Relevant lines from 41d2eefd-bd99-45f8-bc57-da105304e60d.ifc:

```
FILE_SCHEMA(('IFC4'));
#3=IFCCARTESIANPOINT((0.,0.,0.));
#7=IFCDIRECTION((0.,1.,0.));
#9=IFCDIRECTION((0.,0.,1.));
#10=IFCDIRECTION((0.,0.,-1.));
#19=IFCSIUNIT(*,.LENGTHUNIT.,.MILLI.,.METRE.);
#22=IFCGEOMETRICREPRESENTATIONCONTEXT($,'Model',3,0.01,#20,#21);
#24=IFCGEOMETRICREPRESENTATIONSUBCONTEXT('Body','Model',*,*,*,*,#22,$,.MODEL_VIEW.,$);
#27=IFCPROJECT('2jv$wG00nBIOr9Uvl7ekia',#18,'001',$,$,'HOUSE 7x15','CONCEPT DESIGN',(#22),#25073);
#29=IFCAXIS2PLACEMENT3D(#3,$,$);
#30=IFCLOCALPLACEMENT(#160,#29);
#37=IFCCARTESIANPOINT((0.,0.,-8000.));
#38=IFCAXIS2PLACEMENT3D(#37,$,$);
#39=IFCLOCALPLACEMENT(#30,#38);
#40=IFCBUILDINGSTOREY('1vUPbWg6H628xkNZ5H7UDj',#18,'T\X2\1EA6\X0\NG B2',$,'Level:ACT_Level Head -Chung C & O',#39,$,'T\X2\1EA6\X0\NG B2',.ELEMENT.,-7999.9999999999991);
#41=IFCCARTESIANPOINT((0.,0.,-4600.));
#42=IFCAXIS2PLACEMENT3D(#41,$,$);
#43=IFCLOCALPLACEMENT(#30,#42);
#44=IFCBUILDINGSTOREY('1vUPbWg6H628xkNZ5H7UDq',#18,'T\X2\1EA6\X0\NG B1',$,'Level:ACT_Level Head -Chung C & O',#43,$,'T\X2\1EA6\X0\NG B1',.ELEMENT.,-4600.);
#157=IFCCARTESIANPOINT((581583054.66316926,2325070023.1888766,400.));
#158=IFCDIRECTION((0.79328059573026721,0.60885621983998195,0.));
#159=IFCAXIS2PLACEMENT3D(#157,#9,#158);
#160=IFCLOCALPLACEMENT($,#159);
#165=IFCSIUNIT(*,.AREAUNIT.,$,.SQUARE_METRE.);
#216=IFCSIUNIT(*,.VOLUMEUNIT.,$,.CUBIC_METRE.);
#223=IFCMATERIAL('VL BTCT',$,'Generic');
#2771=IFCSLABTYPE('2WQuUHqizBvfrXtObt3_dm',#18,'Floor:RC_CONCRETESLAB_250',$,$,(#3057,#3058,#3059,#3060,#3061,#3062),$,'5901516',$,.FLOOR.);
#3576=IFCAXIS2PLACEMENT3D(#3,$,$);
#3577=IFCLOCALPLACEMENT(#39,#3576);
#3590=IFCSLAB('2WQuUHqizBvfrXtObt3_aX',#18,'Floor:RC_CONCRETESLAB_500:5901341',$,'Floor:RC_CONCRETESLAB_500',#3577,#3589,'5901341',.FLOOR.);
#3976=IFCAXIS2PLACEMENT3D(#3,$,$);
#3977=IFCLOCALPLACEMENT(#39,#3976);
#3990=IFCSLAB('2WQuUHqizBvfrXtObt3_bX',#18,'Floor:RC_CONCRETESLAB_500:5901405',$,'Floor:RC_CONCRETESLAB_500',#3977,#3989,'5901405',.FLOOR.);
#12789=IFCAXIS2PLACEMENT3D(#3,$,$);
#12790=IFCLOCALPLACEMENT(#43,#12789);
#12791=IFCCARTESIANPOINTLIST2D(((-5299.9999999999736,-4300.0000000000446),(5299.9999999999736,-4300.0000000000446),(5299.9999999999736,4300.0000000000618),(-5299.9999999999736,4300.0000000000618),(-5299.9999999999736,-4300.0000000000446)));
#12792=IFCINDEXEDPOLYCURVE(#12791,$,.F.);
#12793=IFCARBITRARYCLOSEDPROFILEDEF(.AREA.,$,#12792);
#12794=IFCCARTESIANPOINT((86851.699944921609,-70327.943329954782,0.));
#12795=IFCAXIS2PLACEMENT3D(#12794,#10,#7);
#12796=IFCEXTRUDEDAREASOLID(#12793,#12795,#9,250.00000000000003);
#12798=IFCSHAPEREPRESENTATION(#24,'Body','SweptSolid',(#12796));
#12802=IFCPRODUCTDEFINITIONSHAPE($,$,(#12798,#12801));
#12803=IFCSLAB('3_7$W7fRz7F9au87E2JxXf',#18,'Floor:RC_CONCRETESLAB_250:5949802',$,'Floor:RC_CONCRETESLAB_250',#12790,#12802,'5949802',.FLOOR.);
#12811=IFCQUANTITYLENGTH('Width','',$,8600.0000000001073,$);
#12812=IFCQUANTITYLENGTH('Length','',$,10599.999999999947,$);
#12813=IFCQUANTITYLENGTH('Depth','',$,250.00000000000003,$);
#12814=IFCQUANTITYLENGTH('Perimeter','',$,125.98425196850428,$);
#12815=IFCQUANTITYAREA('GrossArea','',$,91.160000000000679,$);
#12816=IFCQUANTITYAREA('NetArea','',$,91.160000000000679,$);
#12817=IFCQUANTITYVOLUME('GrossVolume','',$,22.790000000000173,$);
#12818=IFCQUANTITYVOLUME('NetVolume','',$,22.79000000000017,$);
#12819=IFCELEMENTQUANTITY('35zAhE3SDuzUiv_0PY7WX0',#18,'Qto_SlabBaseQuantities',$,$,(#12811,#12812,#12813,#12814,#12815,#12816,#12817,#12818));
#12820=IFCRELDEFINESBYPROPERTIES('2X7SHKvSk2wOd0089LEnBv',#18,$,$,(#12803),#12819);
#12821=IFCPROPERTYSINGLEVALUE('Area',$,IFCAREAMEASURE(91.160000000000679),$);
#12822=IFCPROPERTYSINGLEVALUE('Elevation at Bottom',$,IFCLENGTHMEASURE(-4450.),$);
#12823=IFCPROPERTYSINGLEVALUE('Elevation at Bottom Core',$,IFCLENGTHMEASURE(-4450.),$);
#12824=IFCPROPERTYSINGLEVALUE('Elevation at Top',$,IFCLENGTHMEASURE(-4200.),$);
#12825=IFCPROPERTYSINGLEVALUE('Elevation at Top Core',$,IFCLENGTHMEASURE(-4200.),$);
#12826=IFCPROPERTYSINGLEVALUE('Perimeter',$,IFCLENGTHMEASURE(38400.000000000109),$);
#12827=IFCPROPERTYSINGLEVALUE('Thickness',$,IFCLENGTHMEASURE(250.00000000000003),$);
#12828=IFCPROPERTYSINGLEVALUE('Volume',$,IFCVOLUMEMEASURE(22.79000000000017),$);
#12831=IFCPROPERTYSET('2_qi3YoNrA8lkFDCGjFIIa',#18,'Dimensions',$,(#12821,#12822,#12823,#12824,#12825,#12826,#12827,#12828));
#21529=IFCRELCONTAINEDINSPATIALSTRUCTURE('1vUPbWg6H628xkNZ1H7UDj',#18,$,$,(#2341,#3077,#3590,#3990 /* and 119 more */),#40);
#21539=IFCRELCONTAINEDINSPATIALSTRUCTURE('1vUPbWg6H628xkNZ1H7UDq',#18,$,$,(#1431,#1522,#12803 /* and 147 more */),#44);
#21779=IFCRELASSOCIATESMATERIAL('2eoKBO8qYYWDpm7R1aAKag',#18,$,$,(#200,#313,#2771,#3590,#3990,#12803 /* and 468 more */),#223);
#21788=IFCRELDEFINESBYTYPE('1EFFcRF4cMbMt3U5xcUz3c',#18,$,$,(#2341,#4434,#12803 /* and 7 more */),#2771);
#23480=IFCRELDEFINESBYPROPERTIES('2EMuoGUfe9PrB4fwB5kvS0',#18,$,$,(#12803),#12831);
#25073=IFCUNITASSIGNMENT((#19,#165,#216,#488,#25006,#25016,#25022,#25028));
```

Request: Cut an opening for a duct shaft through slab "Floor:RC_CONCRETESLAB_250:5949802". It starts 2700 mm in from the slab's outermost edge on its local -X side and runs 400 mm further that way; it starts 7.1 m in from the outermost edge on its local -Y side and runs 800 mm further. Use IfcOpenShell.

```python
import numpy as np
import ifcopenshell
import ifcopenshell.api.feature
import ifcopenshell.api.geometry
import ifcopenshell.api.pset
import ifcopenshell.api.root
import ifcopenshell.geom
import ifcopenshell.util.element
import ifcopenshell.util.placement
import ifcopenshell.util.representation
import ifcopenshell.util.shape
import ifcopenshell.util.unit

model = ifcopenshell.open("41d2eefd-bd99-45f8-bc57-da105304e60d.ifc")
unit_scale = ifcopenshell.util.unit.calculate_unit_scale(model)
area_scale = ifcopenshell.util.unit.calculate_unit_scale(model, "AREAUNIT")
volume_scale = ifcopenshell.util.unit.calculate_unit_scale(model, "VOLUMEUNIT")
settings = ifcopenshell.geom.settings()


def volume(element):
    """Net volume in cubic metres, openings subtracted."""
    shape = ifcopenshell.geom.create_shape(settings, element)
    return ifcopenshell.util.shape.get_volume(shape.geometry)


slab = model.by_guid("3_7$W7fRz7F9au87E2JxXf")
before = volume(slab)

# Extent in the slab's own axes, in metres. The edges named are its -X and -Y sides.
slab_shape = ifcopenshell.geom.create_shape(settings, slab)
vertices = ifcopenshell.util.shape.get_vertices(slab_shape.geometry)
x_min, y_min, bottom = vertices.min(axis=0)
top = vertices[:, 2].max()

opening = ifcopenshell.api.root.create_entity(model, ifc_class="IfcOpeningElement", name="Duct shaft opening", predefined_type="OPENING")
context = ifcopenshell.util.representation.get_context(model, "Model", "Body", "MODEL_VIEW")
width, depth = 0.4, 0.8
outline = [(0.0, 0.0), (width, 0.0), (width, depth), (0.0, depth), (0.0, 0.0)]
# Overshoot both faces by 50 mm so the cut is clean.
shape = ifcopenshell.api.geometry.add_slab_representation(
    model, context=context, depth=top - bottom + 0.1, polyline=outline
)
ifcopenshell.api.geometry.assign_representation(model, product=opening, representation=shape)

matrix = ifcopenshell.util.placement.get_local_placement(slab.ObjectPlacement)
matrix[:, 3] = matrix @ np.append(np.array([x_min + 2.7, y_min + 7.1, bottom - 0.05]) / unit_scale, 1.0)
ifcopenshell.api.geometry.edit_object_placement(model, product=opening, matrix=matrix, is_si=False)
ifcopenshell.api.feature.add_feature(model, feature=opening, element=slab)

after = volume(slab)

# Update the slab's stored quantities.
qto = model.by_id(ifcopenshell.util.element.get_pset(slab, "Qto_SlabBaseQuantities", should_inherit=False)["id"])
ifcopenshell.api.pset.edit_qto(model, qto=qto, properties={
    "NetArea": after / (top - bottom) / area_scale,
    "NetVolume": after / volume_scale,
})
pset = model.by_id(ifcopenshell.util.element.get_pset(slab, "Dimensions", should_inherit=False)["id"])
ifcopenshell.api.pset.edit_pset(model, pset=pset, properties={
    "Area": model.create_entity("IfcAreaMeasure", after / (top - bottom) / area_scale),
    "Volume": model.create_entity("IfcVolumeMeasure", after / volume_scale),
})

print(f"slab volume {before:.3f} -> {after:.3f} m3")

model.write("41d2eefd-bd99-45f8-bc57-da105304e60d_edited.ifc")
```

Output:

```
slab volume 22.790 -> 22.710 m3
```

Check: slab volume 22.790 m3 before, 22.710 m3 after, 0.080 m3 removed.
